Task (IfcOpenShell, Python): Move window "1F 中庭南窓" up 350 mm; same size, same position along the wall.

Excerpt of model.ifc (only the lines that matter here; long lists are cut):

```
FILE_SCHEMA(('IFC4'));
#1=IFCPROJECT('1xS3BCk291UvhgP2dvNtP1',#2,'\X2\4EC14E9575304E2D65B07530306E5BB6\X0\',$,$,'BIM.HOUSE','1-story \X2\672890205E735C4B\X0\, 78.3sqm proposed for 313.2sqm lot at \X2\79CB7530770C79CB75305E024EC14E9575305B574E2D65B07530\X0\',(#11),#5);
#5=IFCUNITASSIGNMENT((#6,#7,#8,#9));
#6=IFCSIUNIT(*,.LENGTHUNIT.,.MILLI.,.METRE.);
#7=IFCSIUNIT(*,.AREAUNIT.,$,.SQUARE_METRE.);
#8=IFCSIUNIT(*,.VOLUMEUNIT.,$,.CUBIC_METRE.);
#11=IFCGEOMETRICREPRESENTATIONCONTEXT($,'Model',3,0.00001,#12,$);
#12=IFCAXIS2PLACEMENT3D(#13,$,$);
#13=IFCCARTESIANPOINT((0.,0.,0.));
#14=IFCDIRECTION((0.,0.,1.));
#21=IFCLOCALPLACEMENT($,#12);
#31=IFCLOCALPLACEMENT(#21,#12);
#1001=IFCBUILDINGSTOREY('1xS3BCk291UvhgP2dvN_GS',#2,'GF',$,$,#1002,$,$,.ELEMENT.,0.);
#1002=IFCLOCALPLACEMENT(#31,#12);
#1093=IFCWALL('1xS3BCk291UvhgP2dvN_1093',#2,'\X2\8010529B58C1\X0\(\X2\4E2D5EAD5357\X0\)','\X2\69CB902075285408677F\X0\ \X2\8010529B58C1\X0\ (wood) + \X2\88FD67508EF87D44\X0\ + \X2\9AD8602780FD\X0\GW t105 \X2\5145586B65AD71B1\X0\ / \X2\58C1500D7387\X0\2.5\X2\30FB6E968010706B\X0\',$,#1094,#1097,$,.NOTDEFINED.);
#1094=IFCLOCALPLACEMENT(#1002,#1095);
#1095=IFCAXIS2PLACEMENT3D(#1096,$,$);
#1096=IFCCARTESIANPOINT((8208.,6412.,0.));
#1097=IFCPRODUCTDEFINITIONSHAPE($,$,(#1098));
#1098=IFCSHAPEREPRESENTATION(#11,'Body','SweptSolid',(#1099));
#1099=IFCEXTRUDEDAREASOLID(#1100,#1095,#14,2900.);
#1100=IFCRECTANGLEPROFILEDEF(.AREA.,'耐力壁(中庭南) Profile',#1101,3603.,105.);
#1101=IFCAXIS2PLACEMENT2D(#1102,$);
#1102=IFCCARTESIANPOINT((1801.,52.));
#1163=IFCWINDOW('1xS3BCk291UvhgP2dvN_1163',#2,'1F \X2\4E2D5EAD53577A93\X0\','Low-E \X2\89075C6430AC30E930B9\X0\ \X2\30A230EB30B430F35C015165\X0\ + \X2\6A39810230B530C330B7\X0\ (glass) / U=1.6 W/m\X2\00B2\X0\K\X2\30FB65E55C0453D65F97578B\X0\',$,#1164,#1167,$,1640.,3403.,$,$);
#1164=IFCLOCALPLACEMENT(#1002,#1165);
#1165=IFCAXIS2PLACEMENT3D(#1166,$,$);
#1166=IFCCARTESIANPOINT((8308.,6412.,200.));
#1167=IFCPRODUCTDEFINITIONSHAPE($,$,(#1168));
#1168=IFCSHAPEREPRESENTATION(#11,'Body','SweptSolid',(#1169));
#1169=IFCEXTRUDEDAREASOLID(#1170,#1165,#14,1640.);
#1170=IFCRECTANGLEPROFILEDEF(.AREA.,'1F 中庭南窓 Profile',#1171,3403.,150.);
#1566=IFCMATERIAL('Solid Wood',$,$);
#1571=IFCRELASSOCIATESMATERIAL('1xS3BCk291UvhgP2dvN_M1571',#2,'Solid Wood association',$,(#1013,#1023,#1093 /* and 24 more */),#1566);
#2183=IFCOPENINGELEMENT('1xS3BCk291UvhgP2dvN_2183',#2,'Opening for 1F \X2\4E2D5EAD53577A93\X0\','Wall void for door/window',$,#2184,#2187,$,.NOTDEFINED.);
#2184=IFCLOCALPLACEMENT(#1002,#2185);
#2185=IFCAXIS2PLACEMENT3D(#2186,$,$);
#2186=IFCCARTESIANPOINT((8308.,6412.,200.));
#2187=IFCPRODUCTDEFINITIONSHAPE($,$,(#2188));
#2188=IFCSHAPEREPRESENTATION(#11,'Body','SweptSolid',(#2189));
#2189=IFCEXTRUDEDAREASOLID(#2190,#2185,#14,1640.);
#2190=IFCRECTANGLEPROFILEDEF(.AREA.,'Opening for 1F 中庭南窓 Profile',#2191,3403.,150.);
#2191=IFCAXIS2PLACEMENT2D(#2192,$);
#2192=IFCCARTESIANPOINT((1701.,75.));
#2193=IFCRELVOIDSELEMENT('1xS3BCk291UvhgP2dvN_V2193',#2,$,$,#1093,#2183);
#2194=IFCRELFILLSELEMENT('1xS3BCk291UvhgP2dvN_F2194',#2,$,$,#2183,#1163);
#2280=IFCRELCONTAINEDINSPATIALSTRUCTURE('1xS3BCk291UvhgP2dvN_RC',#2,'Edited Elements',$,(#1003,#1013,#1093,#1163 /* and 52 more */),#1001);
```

```python
import numpy as np
import ifcopenshell
import ifcopenshell.api.geometry
import ifcopenshell.util.placement
import ifcopenshell.util.unit

model = ifcopenshell.open("model.ifc")
unit_scale = ifcopenshell.util.unit.calculate_unit_scale(model)

window = model.by_id(1163)
opening = window.FillsVoids[0].RelatingOpeningElement
dz = 0.35 / unit_scale

shift = np.array([0.0, 0.0, dz])
# The window is not placed relative to its opening, so move both.
for product in (opening, window):
    matrix = ifcopenshell.util.placement.get_local_placement(product.ObjectPlacement)
    matrix[:3, 3] += shift
    ifcopenshell.api.geometry.edit_object_placement(model, product=product, matrix=matrix, is_si=False)

print(f"moved by {dz * unit_scale:+.3f} m")

model.write("model_rev.ifc")
```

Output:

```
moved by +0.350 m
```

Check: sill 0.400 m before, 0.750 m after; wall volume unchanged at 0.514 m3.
